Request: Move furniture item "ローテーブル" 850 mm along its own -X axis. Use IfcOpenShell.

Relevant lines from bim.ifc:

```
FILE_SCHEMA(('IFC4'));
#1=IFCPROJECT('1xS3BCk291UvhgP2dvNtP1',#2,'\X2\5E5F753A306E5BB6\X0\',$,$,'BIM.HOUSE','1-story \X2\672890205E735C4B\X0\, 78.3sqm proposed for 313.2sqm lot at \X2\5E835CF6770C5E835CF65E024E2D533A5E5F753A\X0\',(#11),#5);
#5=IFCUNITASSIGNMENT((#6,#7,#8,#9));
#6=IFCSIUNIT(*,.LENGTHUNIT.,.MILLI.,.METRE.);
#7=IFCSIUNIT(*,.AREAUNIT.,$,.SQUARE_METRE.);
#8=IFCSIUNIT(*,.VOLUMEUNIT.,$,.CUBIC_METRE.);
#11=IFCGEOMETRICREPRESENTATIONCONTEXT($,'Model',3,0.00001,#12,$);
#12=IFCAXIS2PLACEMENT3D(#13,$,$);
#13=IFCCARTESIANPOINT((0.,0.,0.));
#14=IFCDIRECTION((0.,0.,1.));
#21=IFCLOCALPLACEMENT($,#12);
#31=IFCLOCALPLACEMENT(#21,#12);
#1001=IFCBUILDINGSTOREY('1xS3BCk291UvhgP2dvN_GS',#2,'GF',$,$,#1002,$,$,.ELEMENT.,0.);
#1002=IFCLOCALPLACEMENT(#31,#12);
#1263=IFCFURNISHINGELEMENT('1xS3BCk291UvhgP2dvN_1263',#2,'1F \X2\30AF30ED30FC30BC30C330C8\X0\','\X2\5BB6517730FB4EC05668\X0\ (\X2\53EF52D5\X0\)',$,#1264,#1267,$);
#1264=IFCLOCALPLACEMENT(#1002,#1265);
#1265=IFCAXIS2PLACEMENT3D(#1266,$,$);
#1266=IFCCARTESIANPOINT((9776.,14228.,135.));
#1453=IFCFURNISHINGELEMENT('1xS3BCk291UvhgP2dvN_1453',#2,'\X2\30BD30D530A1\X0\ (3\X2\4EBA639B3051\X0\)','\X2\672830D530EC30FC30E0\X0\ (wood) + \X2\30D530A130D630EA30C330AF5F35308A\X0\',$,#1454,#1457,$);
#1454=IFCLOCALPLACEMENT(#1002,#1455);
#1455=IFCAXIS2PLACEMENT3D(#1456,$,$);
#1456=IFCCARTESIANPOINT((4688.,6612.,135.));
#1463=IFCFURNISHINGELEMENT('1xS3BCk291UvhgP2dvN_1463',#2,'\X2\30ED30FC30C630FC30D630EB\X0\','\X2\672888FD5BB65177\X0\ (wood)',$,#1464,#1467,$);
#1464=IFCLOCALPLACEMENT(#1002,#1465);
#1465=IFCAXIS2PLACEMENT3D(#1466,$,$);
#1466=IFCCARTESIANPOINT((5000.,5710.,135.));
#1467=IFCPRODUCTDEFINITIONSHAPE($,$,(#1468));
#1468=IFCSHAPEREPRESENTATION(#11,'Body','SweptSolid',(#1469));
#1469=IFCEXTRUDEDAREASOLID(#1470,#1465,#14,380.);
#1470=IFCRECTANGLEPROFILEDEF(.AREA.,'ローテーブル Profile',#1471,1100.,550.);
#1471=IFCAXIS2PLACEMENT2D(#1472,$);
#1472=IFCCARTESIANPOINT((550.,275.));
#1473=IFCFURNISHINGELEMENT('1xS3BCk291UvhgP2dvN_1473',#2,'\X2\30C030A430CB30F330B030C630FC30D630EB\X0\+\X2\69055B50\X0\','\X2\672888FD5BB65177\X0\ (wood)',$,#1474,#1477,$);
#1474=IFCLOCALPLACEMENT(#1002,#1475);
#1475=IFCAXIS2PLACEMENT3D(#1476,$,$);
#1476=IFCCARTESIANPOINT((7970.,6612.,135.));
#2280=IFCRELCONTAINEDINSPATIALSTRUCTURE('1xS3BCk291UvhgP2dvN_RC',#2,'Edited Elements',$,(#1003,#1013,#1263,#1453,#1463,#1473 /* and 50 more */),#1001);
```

```python
import ifcopenshell
import ifcopenshell.api.geometry
import ifcopenshell.util.placement

model = ifcopenshell.open("bim.ifc")

item = model.by_guid("1xS3BCk291UvhgP2dvN_1463")
matrix = ifcopenshell.util.placement.get_local_placement(item.ObjectPlacement)
matrix[:3, 3] -= matrix[:3, 0] * 850.0
ifcopenshell.api.geometry.edit_object_placement(model, product=item, matrix=matrix, is_si=False)

print(ifcopenshell.util.placement.get_local_placement(item.ObjectPlacement).round(3) + 0.0)

model.write("bim_edited.ifc")
```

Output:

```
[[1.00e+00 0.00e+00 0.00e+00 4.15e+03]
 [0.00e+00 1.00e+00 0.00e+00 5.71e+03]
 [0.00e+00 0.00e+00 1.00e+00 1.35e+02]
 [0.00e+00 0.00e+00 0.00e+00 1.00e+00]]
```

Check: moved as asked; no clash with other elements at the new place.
